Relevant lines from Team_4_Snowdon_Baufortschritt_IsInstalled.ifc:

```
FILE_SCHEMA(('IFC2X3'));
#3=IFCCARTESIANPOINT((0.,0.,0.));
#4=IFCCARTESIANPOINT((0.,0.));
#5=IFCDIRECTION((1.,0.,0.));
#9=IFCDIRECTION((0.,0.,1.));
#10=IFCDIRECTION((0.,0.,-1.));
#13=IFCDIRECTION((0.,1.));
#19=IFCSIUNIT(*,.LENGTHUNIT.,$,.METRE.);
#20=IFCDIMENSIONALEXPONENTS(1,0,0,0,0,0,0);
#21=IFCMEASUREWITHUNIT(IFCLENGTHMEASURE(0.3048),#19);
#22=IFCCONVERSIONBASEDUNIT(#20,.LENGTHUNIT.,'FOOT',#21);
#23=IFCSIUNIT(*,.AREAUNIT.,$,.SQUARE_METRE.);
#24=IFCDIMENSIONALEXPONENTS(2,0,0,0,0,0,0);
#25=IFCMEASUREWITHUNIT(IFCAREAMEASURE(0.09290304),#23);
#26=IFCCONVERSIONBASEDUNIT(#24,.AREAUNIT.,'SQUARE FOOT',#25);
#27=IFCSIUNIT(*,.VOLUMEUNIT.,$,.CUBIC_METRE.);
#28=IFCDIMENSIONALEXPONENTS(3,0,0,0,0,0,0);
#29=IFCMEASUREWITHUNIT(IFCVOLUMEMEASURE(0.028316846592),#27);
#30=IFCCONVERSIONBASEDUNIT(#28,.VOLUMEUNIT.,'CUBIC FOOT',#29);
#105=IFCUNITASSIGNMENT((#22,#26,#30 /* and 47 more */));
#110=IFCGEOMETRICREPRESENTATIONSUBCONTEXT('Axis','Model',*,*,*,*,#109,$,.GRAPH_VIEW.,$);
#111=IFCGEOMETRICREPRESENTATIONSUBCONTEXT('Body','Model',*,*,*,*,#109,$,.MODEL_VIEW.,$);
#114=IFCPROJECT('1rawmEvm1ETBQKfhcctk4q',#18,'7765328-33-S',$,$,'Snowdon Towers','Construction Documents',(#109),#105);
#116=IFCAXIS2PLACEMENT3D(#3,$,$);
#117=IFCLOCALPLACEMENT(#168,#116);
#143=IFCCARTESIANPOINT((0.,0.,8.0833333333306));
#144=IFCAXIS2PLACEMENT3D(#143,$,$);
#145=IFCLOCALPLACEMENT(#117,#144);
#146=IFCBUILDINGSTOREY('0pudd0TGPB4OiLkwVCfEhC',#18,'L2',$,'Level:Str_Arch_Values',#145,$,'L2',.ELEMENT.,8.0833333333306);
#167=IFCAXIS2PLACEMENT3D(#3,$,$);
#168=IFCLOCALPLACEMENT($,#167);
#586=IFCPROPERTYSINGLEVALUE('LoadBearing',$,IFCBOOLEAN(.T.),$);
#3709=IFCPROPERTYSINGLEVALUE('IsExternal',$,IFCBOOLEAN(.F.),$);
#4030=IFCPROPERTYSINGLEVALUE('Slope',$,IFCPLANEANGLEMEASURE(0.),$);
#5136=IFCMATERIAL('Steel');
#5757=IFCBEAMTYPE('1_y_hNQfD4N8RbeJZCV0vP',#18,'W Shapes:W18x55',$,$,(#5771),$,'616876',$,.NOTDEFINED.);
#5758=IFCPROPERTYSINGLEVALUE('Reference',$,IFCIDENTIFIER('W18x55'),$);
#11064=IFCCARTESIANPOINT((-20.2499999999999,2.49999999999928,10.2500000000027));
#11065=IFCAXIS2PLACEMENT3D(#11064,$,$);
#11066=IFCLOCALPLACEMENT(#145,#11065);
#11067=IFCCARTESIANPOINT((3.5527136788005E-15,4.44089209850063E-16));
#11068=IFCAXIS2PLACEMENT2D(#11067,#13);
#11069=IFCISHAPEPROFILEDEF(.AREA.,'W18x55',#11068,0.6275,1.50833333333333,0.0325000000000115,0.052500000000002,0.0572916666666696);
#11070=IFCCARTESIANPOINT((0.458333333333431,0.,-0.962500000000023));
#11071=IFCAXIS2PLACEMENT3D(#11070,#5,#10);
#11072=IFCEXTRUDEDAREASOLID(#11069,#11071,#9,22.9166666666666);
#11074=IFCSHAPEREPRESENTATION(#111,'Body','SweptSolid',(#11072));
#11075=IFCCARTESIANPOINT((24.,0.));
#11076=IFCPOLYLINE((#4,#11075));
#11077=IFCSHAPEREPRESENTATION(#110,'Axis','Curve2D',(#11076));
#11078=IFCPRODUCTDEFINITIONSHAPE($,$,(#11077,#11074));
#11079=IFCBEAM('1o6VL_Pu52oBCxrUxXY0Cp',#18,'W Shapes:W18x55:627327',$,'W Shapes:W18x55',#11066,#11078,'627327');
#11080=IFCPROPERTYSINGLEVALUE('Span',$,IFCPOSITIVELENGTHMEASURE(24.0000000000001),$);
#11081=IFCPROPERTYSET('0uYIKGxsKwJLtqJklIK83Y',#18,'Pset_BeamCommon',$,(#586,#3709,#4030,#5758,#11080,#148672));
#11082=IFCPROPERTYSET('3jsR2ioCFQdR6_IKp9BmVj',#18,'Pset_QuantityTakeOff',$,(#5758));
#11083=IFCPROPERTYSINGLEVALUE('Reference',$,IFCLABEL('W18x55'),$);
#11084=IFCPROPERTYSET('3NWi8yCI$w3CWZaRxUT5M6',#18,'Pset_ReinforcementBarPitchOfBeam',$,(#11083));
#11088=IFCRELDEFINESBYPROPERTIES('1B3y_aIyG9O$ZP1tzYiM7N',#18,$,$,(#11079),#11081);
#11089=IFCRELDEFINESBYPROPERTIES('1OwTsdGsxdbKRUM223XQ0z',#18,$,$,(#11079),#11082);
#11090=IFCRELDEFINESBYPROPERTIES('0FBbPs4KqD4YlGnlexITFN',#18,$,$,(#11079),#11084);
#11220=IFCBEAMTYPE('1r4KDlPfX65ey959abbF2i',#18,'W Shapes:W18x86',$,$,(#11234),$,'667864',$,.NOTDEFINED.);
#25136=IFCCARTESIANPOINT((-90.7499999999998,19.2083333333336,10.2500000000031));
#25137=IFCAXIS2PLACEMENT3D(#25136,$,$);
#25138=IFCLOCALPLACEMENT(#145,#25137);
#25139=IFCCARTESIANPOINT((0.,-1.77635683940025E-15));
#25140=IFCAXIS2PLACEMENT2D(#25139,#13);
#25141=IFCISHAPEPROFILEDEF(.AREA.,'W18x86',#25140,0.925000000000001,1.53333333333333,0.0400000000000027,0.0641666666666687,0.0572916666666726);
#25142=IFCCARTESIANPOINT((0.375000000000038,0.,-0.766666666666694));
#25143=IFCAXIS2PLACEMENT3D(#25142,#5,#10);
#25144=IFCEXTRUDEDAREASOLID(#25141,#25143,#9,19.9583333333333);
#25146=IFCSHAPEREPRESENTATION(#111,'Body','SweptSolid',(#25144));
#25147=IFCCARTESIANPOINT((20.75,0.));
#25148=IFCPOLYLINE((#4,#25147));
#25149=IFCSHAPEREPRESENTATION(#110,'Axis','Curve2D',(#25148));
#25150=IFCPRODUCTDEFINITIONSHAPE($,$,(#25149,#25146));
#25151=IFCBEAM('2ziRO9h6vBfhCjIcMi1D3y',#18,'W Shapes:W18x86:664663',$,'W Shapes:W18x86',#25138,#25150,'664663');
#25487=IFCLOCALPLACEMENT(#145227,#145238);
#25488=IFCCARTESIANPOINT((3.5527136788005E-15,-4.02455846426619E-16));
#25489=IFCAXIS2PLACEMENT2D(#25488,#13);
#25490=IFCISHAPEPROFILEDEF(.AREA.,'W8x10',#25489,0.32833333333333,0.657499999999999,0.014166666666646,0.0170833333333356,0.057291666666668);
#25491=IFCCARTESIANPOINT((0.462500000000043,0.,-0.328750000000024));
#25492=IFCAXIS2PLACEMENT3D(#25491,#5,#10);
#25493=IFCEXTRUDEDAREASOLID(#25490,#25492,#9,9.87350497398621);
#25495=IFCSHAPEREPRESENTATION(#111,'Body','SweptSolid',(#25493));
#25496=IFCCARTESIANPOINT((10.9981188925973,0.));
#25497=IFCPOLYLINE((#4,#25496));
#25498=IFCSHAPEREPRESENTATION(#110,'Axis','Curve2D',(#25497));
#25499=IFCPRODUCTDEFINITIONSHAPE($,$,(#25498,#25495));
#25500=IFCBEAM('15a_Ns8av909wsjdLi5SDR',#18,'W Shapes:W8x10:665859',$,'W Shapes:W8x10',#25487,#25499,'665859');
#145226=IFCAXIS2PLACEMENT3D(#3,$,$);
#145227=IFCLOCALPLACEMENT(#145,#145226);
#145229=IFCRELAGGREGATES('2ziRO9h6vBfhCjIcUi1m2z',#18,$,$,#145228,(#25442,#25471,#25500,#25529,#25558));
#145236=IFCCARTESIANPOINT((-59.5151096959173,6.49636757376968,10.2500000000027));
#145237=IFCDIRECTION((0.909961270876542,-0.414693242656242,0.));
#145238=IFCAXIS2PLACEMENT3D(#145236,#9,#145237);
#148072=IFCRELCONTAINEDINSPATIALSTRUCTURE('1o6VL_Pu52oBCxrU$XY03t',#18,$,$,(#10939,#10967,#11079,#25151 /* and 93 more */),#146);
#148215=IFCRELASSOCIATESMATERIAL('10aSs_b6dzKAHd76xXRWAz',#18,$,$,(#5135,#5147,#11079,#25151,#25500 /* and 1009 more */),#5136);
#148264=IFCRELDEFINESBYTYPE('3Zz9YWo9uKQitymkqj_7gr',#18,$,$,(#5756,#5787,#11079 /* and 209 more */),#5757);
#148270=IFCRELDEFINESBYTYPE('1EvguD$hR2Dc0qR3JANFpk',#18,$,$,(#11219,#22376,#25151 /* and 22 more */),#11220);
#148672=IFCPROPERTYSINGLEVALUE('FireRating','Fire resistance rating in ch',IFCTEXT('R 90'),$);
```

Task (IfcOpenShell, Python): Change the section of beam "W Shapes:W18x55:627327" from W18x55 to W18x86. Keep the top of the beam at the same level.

```python
import ifcopenshell
import ifcopenshell.api.pset
import ifcopenshell.api.type
import ifcopenshell.util.element
import ifcopenshell.util.representation

model = ifcopenshell.open("Team_4_Snowdon_Baufortschritt_IsInstalled.ifc")

member = model.by_guid("1o6VL_Pu52oBCxrUxXY0Cp")
source = next(p for p in model.by_type("IfcIShapeProfileDef") if p.ProfileName == "W18x86")

body = ifcopenshell.util.representation.get_representation(member, "Model", "Body")
solid = body.Items[0]
old_profile = solid.SweptArea

# Copy the section's sizes but keep this member's own profile position.
profile = ifcopenshell.util.element.copy(model, source)
# Profiles are centred, so shift by half the change in depth to hold the top.
shift = (old_profile.OverallDepth - profile.OverallDepth) / 2
x, y = old_profile.Position.Location.Coordinates
up = (-1.0, 0.0)  # upwards, in the solid's own plane
location = model.createIfcCartesianPoint((x + up[0] * shift, y + up[1] * shift))
profile.Position = model.createIfcAxis2Placement2D(location, old_profile.Position.RefDirection)
solid.SweptArea = profile
if not model.get_total_inverses(old_profile):
    ifcopenshell.util.element.remove_deep2(model, old_profile)

new_type = model.by_id(11220)
ifcopenshell.api.type.assign_type(
    model, related_objects=[member], relating_type=new_type, should_map_representations=False
)
member.Name = member.Name.replace("W18x55", "W18x86")
member.ObjectType = "W Shapes:W18x86"
pset = model.by_id(ifcopenshell.util.element.get_pset(member, "Pset_BeamCommon", should_inherit=False)["id"])
ifcopenshell.api.pset.edit_pset(model, pset=pset, properties={"Reference": "W18x86"})
pset = model.by_id(ifcopenshell.util.element.get_pset(member, "Pset_QuantityTakeOff", should_inherit=False)["id"])
ifcopenshell.api.pset.edit_pset(model, pset=pset, properties={"Reference": "W18x86"})
pset = model.by_id(ifcopenshell.util.element.get_pset(member, "Pset_ReinforcementBarPitchOfBeam", should_inherit=False)["id"])
ifcopenshell.api.pset.edit_pset(model, pset=pset, properties={"Reference": "W18x86"})

print(solid.SweptArea)

model.write("Team_4_Snowdon_Baufortschritt_IsInstalled_rev.ifc")
```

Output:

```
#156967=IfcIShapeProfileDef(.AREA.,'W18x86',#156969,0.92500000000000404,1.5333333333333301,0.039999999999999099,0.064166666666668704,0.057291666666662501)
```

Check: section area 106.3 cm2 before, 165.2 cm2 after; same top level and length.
